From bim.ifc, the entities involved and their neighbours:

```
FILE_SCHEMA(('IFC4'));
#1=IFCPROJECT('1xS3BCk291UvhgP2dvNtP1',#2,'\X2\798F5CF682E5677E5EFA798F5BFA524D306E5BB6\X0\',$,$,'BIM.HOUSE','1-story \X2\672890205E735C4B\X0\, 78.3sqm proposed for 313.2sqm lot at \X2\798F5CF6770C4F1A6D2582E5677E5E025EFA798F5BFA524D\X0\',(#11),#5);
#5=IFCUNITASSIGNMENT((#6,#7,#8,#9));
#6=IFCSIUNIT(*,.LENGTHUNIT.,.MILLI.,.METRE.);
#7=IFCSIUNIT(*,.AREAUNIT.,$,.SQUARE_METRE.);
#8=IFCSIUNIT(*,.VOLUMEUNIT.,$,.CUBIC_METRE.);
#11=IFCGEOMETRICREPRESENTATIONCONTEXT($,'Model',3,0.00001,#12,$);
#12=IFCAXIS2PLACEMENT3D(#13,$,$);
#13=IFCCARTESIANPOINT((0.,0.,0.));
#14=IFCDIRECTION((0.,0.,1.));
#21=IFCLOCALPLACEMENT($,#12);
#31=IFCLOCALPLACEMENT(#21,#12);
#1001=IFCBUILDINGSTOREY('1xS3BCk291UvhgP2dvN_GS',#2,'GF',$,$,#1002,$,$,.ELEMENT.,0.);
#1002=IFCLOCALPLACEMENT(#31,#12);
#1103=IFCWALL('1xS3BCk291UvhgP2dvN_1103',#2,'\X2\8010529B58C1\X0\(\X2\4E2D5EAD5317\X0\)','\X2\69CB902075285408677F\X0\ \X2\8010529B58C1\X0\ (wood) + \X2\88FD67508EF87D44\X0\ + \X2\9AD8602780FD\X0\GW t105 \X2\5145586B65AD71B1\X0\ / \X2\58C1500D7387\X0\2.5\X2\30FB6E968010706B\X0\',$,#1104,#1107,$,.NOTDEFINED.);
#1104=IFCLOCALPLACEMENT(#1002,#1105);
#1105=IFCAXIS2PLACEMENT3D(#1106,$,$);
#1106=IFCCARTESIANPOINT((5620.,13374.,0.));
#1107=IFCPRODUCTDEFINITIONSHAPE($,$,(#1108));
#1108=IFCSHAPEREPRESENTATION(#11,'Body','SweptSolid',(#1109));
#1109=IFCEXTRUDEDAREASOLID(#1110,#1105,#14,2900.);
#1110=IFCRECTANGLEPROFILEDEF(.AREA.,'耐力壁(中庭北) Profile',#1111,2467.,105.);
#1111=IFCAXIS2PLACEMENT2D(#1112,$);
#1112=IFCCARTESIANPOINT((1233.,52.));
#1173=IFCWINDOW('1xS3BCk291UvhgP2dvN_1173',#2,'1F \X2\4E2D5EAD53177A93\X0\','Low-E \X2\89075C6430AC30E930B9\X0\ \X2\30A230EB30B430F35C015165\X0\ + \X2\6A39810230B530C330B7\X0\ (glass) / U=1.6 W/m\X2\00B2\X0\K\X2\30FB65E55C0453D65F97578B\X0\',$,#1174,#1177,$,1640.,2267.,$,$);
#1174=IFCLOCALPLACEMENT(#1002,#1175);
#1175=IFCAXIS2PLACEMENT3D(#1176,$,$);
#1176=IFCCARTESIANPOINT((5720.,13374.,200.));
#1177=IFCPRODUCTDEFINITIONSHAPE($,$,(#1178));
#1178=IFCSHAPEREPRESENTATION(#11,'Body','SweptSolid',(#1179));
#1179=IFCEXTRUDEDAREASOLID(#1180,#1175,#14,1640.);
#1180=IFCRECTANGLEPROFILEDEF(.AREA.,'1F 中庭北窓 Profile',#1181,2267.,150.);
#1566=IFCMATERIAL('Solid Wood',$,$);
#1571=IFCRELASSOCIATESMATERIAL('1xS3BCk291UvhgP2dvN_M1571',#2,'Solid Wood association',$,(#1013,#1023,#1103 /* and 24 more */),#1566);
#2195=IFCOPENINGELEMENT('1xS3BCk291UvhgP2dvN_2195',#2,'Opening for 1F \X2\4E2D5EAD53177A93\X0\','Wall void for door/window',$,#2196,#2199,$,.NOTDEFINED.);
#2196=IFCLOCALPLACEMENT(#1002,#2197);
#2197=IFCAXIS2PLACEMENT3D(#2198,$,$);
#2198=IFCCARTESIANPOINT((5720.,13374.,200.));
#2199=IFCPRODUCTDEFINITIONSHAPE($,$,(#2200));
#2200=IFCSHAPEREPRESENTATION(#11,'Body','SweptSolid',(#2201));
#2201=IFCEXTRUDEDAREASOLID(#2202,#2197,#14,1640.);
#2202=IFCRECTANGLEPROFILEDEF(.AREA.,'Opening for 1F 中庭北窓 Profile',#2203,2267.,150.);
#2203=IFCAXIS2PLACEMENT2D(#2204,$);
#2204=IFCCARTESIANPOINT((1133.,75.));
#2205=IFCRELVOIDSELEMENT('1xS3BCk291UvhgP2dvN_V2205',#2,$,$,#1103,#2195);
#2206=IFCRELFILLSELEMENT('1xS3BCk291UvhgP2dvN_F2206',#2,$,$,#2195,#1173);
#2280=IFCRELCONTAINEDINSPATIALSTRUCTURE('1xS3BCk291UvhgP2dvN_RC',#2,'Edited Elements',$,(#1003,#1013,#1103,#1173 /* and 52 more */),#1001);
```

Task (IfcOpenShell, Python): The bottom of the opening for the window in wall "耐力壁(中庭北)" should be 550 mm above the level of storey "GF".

```python
import numpy as np
import ifcopenshell
import ifcopenshell.api.geometry
import ifcopenshell.geom
import ifcopenshell.util.element
import ifcopenshell.util.placement
import ifcopenshell.util.shape
import ifcopenshell.util.unit

model = ifcopenshell.open("bim.ifc")
unit_scale = ifcopenshell.util.unit.calculate_unit_scale(model)

window = model.by_guid("1xS3BCk291UvhgP2dvN_1173")
opening = window.FillsVoids[0].RelatingOpeningElement
storey = ifcopenshell.util.element.get_container(window, ifc_class="IfcBuildingStorey")
level = ifcopenshell.util.placement.get_local_placement(storey.ObjectPlacement)[2, 3]

# The opening's origin need not be at the sill, so measure its lowest point.
shape = ifcopenshell.geom.create_shape(ifcopenshell.geom.settings(), opening)
bottom = ifcopenshell.util.shape.get_shape_bottom_elevation(shape, shape.geometry) / unit_scale
dz = level + 0.55 / unit_scale - bottom

shift = np.array([0.0, 0.0, dz])
# The window is not placed relative to its opening, so move both.
for product in (opening, window):
    matrix = ifcopenshell.util.placement.get_local_placement(product.ObjectPlacement)
    matrix[:3, 3] += shift
    ifcopenshell.api.geometry.edit_object_placement(model, product=product, matrix=matrix, is_si=False)

print(f"moved by {dz * unit_scale:+.3f} m")

model.write("bim_v2.ifc")
```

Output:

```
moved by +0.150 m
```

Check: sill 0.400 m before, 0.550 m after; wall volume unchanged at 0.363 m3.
